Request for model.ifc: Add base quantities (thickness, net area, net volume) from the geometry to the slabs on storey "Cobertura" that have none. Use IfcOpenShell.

First a look at what the model holds.

```python
import ifcopenshell
import ifcopenshell.util.element
import ifcopenshell.util.unit

model = ifcopenshell.open("model.ifc")
print(model.schema)
for unit_type in ("LENGTHUNIT", "AREAUNIT", "VOLUMEUNIT"):
    print(unit_type, ifcopenshell.util.unit.calculate_unit_scale(model, unit_type))
storey = next(s for s in model.by_type("IfcBuildingStorey") if s.Name == "Cobertura")
slabs = [e for e in ifcopenshell.util.element.get_decomposition(storey) if e.is_a("IfcSlab")]
for e in sorted(slabs, key=lambda e: e.id()):
    print(e.id(), e.is_a(), e.Name, list(ifcopenshell.util.element.get_psets(e, qtos_only=True)), sep=" | ")
```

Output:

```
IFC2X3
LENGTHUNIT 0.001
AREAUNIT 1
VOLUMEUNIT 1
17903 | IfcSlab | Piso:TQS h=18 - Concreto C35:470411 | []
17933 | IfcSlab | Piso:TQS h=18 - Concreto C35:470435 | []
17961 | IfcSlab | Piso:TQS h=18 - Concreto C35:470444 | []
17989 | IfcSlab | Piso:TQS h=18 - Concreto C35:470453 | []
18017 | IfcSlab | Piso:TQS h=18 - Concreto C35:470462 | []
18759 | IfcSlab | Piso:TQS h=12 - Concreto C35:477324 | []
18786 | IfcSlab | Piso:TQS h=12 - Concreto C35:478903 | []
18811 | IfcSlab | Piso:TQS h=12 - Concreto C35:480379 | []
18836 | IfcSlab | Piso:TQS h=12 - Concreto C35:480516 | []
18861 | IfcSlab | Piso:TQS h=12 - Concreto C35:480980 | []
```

```python
import ifcopenshell
import ifcopenshell.api.pset
import ifcopenshell.geom
import ifcopenshell.util.element
import ifcopenshell.util.shape
import ifcopenshell.util.unit

model = ifcopenshell.open("model.ifc")
unit_scale = ifcopenshell.util.unit.calculate_unit_scale(model)
area_scale = ifcopenshell.util.unit.calculate_unit_scale(model, "AREAUNIT")
volume_scale = ifcopenshell.util.unit.calculate_unit_scale(model, "VOLUMEUNIT")
settings = ifcopenshell.geom.settings()

storey = next(s for s in model.by_type("IfcBuildingStorey") if s.Name == "Cobertura")
slabs = [e for e in ifcopenshell.util.element.get_decomposition(storey) if e.is_a("IfcSlab")]

for e in sorted(slabs, key=lambda e: e.id()):
    if ifcopenshell.util.element.get_psets(e, qtos_only=True, should_inherit=False):
        continue
    # Geometry comes back in metres, in the element's own axes.
    shape = ifcopenshell.geom.create_shape(settings, e)
    values = {
        "Width": ifcopenshell.util.shape.get_z(shape.geometry) / unit_scale,
        "NetArea": ifcopenshell.util.shape.get_footprint_area(shape.geometry) / area_scale,
        "NetVolume": ifcopenshell.util.shape.get_volume(shape.geometry) / volume_scale,
    }
    qto = ifcopenshell.api.pset.add_qto(model, product=e, name="BaseQuantities")
    ifcopenshell.api.pset.edit_qto(model, qto=qto, properties=values)
    print(e.id(), {k: round(v, 3) for k, v in values.items()})

model.write("model-out.ifc")
```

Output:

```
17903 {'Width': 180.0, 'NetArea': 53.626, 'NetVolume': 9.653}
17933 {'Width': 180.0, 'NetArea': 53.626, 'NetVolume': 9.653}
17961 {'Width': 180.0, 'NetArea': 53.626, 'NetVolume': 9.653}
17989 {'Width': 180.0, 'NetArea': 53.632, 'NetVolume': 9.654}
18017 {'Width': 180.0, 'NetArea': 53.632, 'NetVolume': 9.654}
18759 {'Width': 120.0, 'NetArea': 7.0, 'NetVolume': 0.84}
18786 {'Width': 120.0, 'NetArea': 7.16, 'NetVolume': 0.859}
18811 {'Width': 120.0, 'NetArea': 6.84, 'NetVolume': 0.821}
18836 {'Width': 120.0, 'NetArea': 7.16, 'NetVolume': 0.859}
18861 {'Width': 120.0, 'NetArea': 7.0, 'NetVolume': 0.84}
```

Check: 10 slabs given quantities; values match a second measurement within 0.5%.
